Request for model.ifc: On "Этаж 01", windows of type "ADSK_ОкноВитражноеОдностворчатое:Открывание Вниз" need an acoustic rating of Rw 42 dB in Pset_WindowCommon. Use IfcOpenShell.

First a look at what the model holds.

```python
import ifcopenshell
import ifcopenshell.util.element

model = ifcopenshell.open("model.ifc")
print(model.schema)
storey = next(s for s in model.by_type("IfcBuildingStorey") if s.Name == "Этаж 01")
windows = [e for e in ifcopenshell.util.element.get_decomposition(storey) if e.is_a("IfcWindow")]
seen = {}
for e in windows:
    element_type = ifcopenshell.util.element.get_type(e)
    key = (element_type.Name if element_type != e and element_type else None, ifcopenshell.util.element.get_pset(e, "Pset_WindowCommon", "AcousticRating"))
    seen[key] = seen.get(key, 0) + 1
for (name, value), count in sorted(seen.items(), key=str):
    print(count, "x", name, "|", value)
```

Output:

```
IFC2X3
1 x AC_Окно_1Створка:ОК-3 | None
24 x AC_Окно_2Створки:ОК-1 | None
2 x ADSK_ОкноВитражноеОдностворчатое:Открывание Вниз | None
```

```python
import ifcopenshell
import ifcopenshell.api.pset
import ifcopenshell.util.element

model = ifcopenshell.open("model.ifc")

storey = next(s for s in model.by_type("IfcBuildingStorey") if s.Name == "Этаж 01")
windows = [e for e in ifcopenshell.util.element.get_decomposition(storey) if e.is_a("IfcWindow")]

count = 0
for e in windows:
    element_type = ifcopenshell.util.element.get_type(e)
    if element_type in (None, e) or element_type.Name != "ADSK_ОкноВитражноеОдностворчатое:Открывание Вниз":
        continue
    # add_pset returns the element's existing set when there is one.
    pset = ifcopenshell.api.pset.add_pset(model, product=e, name="Pset_WindowCommon")
    ifcopenshell.api.pset.edit_pset(model, pset=pset, properties={"AcousticRating": "Rw 42 dB"})
    count += 1

print(count, "windows updated")

model.write("model-out.ifc")
```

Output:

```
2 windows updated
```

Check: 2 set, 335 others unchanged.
